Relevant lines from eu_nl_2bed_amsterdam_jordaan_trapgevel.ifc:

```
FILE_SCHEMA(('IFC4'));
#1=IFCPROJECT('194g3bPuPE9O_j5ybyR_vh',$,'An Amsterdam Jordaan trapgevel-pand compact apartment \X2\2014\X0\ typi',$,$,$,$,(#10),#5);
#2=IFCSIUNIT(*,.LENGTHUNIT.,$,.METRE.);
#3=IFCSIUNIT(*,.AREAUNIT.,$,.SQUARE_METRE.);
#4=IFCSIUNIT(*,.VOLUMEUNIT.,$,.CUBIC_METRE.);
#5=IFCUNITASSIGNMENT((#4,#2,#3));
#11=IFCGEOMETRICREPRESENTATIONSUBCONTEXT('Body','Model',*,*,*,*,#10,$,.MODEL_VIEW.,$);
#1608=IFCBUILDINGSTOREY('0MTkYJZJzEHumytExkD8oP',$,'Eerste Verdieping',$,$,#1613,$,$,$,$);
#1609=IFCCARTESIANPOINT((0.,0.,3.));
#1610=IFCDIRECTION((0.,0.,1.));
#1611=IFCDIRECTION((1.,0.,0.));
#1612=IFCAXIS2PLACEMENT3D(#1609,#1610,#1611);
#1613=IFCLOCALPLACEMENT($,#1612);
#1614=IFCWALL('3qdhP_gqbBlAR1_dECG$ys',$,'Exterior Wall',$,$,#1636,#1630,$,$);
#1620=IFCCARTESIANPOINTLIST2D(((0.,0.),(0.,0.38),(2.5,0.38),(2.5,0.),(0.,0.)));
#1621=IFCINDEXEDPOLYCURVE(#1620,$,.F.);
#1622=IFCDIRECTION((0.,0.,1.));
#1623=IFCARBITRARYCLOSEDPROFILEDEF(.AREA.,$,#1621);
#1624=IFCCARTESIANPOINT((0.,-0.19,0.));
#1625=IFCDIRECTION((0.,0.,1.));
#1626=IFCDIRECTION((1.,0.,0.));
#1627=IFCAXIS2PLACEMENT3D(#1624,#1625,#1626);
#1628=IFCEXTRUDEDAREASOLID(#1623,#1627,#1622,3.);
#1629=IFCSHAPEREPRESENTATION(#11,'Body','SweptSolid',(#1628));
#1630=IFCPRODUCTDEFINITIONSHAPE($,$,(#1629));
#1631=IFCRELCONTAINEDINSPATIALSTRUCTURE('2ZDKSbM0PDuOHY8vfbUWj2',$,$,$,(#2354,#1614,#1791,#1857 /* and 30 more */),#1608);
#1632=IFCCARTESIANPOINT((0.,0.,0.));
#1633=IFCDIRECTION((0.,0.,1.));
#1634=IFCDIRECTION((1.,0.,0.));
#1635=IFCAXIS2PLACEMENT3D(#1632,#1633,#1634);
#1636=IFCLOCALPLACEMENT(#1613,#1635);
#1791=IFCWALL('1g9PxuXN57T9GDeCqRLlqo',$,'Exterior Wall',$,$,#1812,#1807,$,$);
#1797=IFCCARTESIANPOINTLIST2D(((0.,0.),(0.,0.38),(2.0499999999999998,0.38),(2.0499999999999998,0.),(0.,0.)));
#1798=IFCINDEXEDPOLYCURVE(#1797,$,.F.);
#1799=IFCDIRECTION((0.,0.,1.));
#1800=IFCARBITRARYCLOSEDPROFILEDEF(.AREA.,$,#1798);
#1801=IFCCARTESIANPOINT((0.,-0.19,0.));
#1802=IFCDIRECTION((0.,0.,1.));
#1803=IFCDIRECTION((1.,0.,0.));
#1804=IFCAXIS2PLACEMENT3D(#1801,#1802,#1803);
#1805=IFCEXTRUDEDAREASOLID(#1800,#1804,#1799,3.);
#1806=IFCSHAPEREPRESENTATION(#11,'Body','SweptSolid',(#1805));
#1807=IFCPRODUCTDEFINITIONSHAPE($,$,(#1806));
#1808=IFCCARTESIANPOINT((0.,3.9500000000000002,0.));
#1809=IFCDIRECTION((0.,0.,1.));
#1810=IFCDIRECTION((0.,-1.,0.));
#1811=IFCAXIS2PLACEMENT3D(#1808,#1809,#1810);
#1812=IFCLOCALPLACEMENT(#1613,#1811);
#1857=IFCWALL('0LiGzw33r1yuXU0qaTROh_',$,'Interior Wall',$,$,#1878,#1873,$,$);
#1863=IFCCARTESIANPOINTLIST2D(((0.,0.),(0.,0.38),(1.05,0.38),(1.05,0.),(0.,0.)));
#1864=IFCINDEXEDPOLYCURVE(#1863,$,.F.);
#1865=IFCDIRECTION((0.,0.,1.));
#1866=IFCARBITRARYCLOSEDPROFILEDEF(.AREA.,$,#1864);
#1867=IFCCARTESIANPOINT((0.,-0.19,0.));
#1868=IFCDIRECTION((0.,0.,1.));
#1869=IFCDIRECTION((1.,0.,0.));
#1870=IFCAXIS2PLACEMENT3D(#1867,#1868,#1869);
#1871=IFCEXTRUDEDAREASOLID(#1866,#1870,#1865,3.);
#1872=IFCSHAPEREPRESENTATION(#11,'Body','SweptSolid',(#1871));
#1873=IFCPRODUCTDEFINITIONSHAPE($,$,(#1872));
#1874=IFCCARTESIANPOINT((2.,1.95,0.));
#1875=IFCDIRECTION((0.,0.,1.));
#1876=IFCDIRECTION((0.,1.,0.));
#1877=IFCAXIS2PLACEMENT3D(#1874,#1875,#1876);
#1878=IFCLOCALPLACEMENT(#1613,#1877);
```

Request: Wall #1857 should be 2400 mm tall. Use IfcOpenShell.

```python
import ifcopenshell
import ifcopenshell.geom
import ifcopenshell.util.representation
import ifcopenshell.util.shape
import ifcopenshell.util.unit

model = ifcopenshell.open("eu_nl_2bed_amsterdam_jordaan_trapgevel.ifc")
unit_scale = ifcopenshell.util.unit.calculate_unit_scale(model)
settings = ifcopenshell.geom.settings()


def volume(element):
    """Net volume in cubic metres, openings subtracted."""
    shape = ifcopenshell.geom.create_shape(settings, element)
    return ifcopenshell.util.shape.get_volume(shape.geometry)


wall = model.by_id(1857)
before = volume(wall)

body = ifcopenshell.util.representation.get_representation(wall, "Model", "Body")
solid = body.Items[0]
old_height = solid.Depth
solid.Depth = 2.4 / unit_scale
after = volume(wall)

print(f"height {old_height:g} -> {solid.Depth:g}, volume {before:.3f} -> {after:.3f} m3")

model.write("eu_nl_2bed_amsterdam_jordaan_trapgevel_rev.ifc")
```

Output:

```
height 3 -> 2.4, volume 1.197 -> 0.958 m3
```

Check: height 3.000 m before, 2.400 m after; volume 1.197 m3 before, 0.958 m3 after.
